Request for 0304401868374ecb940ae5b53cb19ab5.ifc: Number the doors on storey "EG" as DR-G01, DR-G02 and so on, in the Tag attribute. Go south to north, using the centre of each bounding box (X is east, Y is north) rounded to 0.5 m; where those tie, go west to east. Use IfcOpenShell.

First a look at what the model holds.

```python
import ifcopenshell
import ifcopenshell.util.element
import ifcopenshell.util.placement

model = ifcopenshell.open("0304401868374ecb940ae5b53cb19ab5.ifc")
print(model.schema)
storey = next(s for s in model.by_type("IfcBuildingStorey") if s.Name == "EG")
doors = [e for e in ifcopenshell.util.element.get_decomposition(storey) if e.is_a("IfcDoor")]
for e in sorted(doors, key=lambda e: e.id()):
    origin = ifcopenshell.util.placement.get_local_placement(e.ObjectPlacement)[:3, 3]
    print(e.id(), e.Tag, e.Name, origin.round(2) + 0.0, sep=" | ")
```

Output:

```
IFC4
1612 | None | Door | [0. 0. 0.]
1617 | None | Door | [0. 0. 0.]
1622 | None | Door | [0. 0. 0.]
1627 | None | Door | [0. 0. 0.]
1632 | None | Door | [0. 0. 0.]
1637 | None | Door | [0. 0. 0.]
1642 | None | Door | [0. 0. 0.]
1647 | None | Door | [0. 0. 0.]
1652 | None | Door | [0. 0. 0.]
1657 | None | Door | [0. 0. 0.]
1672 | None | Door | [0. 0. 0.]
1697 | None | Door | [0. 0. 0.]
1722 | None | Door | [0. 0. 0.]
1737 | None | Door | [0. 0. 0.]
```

```python
import ifcopenshell
import ifcopenshell.geom
import ifcopenshell.util.element
import ifcopenshell.util.shape

model = ifcopenshell.open("0304401868374ecb940ae5b53cb19ab5.ifc")
settings = ifcopenshell.geom.settings()
settings.set("use-world-coords", True)


def centre(element):
    shape = ifcopenshell.geom.create_shape(settings, element)
    return ifcopenshell.util.shape.get_bbox_centroid(shape.geometry)


storey = next(s for s in model.by_type("IfcBuildingStorey") if s.Name == "EG")
doors = [e for e in ifcopenshell.util.element.get_decomposition(storey) if e.is_a("IfcDoor")]

# Insertion points can sit at a corner or the storey origin, so sort by the geometry (in metres).
centres = {e: centre(e) for e in doors}
doors.sort(key=lambda e: (round(centres[e][1] / 0.5), centres[e][0]))

for i, e in enumerate(doors, start=1):
    number = f"DR-G{i:02d}"
    e.Tag = number
    print(e.id(), number)

model.write("0304401868374ecb940ae5b53cb19ab5-out.ifc")
```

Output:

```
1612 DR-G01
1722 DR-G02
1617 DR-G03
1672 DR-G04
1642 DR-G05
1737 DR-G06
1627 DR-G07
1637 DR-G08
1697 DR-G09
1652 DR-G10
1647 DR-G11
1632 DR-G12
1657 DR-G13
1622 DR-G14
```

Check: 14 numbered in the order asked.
